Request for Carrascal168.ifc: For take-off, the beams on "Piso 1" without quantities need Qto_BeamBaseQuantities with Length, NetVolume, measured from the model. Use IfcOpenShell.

First a look at what the model holds.

```python
import ifcopenshell
import ifcopenshell.util.element
import ifcopenshell.util.unit

model = ifcopenshell.open("Carrascal168.ifc")
print(model.schema)
for unit_type in ("LENGTHUNIT", "AREAUNIT", "VOLUMEUNIT"):
    print(unit_type, ifcopenshell.util.unit.calculate_unit_scale(model, unit_type))
storey = next(s for s in model.by_type("IfcBuildingStorey") if s.Name == "Piso 1")
beams = [e for e in ifcopenshell.util.element.get_decomposition(storey) if e.is_a("IfcBeam")]
for e in sorted(beams, key=lambda e: e.id()):
    print(e.id(), e.is_a(), e.Name, list(ifcopenshell.util.element.get_psets(e, qtos_only=True)), sep=" | ")
```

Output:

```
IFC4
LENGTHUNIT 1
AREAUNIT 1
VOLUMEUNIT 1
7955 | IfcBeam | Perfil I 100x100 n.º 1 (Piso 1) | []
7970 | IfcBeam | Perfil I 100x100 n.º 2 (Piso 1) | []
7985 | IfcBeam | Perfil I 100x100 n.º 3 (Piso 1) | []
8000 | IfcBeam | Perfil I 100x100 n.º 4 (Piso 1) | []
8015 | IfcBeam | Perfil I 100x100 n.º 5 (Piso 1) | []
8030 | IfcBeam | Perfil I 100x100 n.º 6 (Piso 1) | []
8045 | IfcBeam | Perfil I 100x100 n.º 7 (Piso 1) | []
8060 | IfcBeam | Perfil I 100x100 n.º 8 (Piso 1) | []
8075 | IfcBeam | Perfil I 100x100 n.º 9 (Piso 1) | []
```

```python
import ifcopenshell
import ifcopenshell.api.pset
import ifcopenshell.geom
import ifcopenshell.util.element
import ifcopenshell.util.shape
import ifcopenshell.util.unit

model = ifcopenshell.open("Carrascal168.ifc")
unit_scale = ifcopenshell.util.unit.calculate_unit_scale(model)
volume_scale = ifcopenshell.util.unit.calculate_unit_scale(model, "VOLUMEUNIT")
settings = ifcopenshell.geom.settings()

storey = next(s for s in model.by_type("IfcBuildingStorey") if s.Name == "Piso 1")
beams = [e for e in ifcopenshell.util.element.get_decomposition(storey) if e.is_a("IfcBeam")]

for e in sorted(beams, key=lambda e: e.id()):
    if ifcopenshell.util.element.get_psets(e, qtos_only=True, should_inherit=False):
        continue
    # Geometry comes back in metres, in the element's own axes.
    shape = ifcopenshell.geom.create_shape(settings, e)
    values = {
        "Length": ifcopenshell.util.shape.get_max_xyz(shape.geometry) / unit_scale,
        "NetVolume": ifcopenshell.util.shape.get_volume(shape.geometry) / volume_scale,
    }
    qto = ifcopenshell.api.pset.add_qto(model, product=e, name="Qto_BeamBaseQuantities")
    ifcopenshell.api.pset.edit_qto(model, qto=qto, properties=values)
    print(e.id(), {k: round(v, 3) for k, v in values.items()})

model.write("Carrascal168_v2.ifc")
```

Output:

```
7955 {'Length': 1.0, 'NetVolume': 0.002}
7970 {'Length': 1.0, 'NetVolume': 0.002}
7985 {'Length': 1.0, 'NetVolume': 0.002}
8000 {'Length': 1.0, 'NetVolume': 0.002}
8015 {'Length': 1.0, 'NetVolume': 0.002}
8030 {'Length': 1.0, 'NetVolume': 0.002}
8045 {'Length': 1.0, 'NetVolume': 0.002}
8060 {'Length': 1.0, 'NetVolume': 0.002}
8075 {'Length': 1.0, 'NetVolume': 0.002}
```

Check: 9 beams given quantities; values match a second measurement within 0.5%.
